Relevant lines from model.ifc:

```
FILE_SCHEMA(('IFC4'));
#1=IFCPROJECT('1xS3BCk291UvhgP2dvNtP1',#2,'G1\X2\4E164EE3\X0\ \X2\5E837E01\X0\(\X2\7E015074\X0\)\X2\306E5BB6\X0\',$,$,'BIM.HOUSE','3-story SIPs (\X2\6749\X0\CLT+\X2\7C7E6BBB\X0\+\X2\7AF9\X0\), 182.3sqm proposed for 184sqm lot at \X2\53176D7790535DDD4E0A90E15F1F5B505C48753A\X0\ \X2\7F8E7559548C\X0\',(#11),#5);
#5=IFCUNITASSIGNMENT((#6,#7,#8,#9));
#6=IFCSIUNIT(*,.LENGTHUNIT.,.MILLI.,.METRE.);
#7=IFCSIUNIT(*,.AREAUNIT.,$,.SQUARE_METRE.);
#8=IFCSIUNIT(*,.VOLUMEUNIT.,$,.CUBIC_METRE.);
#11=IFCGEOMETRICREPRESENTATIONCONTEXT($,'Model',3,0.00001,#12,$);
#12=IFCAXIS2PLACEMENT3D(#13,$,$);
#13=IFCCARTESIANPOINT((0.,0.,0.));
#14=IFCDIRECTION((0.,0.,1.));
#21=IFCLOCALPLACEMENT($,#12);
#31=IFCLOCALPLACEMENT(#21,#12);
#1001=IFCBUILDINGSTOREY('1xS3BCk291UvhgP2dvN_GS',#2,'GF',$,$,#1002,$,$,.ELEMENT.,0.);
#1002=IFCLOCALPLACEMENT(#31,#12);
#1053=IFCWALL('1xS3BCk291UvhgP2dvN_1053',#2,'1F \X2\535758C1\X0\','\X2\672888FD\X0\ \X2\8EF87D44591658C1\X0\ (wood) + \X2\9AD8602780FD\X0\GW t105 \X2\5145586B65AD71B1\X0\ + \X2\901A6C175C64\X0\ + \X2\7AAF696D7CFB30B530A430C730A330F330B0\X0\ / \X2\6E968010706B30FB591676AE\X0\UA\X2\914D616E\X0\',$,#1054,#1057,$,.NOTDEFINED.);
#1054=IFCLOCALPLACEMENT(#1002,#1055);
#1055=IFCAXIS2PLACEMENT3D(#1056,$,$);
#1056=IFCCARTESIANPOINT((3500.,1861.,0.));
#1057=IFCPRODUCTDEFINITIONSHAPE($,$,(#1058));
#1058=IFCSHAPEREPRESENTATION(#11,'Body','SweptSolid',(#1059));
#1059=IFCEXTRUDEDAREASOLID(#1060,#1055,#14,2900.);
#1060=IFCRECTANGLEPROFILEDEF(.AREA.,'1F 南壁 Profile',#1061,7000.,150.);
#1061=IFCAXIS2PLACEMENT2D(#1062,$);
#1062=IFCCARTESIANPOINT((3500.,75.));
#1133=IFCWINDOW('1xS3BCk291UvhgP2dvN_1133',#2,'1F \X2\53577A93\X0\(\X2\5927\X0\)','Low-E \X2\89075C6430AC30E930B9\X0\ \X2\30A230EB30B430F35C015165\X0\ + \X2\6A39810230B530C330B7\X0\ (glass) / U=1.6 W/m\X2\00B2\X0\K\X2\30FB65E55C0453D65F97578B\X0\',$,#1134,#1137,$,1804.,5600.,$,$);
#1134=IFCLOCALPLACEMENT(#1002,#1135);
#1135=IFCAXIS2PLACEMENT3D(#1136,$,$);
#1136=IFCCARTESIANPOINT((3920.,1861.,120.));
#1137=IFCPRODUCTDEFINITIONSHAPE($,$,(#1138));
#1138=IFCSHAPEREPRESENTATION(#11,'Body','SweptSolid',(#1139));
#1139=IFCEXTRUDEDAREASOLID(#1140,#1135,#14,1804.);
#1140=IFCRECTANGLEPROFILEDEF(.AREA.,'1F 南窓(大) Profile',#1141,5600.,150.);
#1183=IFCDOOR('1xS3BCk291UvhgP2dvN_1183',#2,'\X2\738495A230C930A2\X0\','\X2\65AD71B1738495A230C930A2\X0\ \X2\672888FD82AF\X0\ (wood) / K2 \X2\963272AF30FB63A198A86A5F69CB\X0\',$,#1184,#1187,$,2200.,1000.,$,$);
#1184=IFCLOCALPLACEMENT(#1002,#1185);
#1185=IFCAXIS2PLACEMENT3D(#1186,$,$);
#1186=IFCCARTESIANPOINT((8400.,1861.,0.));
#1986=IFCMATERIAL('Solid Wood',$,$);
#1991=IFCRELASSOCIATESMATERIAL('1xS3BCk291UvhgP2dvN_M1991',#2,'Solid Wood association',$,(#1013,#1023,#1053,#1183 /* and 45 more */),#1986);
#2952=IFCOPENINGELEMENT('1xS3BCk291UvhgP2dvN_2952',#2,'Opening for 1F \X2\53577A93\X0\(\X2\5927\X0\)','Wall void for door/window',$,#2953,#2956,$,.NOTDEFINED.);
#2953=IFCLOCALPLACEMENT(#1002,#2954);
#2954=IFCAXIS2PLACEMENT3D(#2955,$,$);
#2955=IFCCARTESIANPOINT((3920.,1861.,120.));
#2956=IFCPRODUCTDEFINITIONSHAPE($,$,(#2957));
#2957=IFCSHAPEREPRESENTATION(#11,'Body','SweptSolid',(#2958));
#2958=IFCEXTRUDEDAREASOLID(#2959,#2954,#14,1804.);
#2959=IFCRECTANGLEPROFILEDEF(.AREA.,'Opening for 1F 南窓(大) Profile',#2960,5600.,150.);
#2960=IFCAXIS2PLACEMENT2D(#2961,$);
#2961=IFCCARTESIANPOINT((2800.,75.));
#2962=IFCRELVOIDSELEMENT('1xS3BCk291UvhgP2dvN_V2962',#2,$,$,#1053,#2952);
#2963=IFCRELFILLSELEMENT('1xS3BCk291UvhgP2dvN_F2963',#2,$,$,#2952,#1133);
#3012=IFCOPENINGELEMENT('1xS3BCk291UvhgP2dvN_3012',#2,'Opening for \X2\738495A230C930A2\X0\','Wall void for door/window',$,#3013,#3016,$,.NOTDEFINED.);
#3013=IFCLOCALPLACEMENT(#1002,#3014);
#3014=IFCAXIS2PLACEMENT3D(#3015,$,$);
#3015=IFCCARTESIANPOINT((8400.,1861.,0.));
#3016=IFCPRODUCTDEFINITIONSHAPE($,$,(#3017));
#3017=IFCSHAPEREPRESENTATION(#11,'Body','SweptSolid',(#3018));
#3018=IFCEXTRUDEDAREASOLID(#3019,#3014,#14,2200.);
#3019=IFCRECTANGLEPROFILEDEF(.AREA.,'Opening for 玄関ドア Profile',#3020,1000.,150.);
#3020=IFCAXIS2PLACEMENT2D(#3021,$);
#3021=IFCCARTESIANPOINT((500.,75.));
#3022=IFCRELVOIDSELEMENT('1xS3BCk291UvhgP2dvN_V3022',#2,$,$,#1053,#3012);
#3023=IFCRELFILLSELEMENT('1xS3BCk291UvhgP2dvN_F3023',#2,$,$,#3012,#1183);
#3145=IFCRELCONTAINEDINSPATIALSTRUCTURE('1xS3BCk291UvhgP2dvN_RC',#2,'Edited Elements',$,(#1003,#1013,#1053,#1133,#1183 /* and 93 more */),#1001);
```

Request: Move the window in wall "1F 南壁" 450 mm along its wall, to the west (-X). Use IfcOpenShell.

```python
import ifcopenshell
import ifcopenshell.api.geometry
import ifcopenshell.util.placement

model = ifcopenshell.open("model.ifc")

window = model.by_guid("1xS3BCk291UvhgP2dvN_1133")
opening = window.FillsVoids[0].RelatingOpeningElement
wall = opening.VoidsElements[0].RelatingBuildingElement

wall_matrix = ifcopenshell.util.placement.get_local_placement(wall.ObjectPlacement)
shift = wall_matrix[:3, 0] * -450.0
before = ifcopenshell.util.placement.get_local_placement(window.ObjectPlacement)[:3, 3].copy()

# The window is not placed relative to its opening, so move both.
for product in (opening, window):
    matrix = ifcopenshell.util.placement.get_local_placement(product.ObjectPlacement)
    matrix[:3, 3] += shift
    ifcopenshell.api.geometry.edit_object_placement(model, product=product, matrix=matrix, is_si=False)

after = ifcopenshell.util.placement.get_local_placement(window.ObjectPlacement)[:3, 3]
print("window moved by", (after - before).round(3) + 0.0)

model.write("model-out.ifc")
```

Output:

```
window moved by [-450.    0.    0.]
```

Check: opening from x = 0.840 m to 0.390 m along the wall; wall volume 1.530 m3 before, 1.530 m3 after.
